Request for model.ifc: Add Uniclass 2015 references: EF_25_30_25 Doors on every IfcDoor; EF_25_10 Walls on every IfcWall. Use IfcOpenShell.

First a look at what the model holds.

```python
import ifcopenshell

model = ifcopenshell.open("model.ifc")
print(model.schema)
print("classifications:", [c.Name for c in model.by_type("IfcClassification")])
for ifc_class in ("IfcDoor", "IfcRoof", "IfcStair", "IfcWall", "IfcWindow"):
    print(ifc_class, len(model.by_type(ifc_class)))
```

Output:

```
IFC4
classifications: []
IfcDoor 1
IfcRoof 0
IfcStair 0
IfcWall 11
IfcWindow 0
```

```python
import ifcopenshell
import ifcopenshell.api.classification

model = ifcopenshell.open("model.ifc")

system = ifcopenshell.api.classification.add_classification(model, classification="Uniclass 2015")

codes = {
    "IfcDoor": ("EF_25_30_25", "Doors"),
    "IfcWall": ("EF_25_10", "Walls"),
}
for ifc_class, (code, name) in codes.items():
    products = model.by_type(ifc_class)
    ifcopenshell.api.classification.add_reference(
        model, products=products, classification=system, identification=code, name=name
    )
    print(code, len(products))

model.write("model_rev.ifc")
```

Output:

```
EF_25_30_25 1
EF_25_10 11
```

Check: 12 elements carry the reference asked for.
